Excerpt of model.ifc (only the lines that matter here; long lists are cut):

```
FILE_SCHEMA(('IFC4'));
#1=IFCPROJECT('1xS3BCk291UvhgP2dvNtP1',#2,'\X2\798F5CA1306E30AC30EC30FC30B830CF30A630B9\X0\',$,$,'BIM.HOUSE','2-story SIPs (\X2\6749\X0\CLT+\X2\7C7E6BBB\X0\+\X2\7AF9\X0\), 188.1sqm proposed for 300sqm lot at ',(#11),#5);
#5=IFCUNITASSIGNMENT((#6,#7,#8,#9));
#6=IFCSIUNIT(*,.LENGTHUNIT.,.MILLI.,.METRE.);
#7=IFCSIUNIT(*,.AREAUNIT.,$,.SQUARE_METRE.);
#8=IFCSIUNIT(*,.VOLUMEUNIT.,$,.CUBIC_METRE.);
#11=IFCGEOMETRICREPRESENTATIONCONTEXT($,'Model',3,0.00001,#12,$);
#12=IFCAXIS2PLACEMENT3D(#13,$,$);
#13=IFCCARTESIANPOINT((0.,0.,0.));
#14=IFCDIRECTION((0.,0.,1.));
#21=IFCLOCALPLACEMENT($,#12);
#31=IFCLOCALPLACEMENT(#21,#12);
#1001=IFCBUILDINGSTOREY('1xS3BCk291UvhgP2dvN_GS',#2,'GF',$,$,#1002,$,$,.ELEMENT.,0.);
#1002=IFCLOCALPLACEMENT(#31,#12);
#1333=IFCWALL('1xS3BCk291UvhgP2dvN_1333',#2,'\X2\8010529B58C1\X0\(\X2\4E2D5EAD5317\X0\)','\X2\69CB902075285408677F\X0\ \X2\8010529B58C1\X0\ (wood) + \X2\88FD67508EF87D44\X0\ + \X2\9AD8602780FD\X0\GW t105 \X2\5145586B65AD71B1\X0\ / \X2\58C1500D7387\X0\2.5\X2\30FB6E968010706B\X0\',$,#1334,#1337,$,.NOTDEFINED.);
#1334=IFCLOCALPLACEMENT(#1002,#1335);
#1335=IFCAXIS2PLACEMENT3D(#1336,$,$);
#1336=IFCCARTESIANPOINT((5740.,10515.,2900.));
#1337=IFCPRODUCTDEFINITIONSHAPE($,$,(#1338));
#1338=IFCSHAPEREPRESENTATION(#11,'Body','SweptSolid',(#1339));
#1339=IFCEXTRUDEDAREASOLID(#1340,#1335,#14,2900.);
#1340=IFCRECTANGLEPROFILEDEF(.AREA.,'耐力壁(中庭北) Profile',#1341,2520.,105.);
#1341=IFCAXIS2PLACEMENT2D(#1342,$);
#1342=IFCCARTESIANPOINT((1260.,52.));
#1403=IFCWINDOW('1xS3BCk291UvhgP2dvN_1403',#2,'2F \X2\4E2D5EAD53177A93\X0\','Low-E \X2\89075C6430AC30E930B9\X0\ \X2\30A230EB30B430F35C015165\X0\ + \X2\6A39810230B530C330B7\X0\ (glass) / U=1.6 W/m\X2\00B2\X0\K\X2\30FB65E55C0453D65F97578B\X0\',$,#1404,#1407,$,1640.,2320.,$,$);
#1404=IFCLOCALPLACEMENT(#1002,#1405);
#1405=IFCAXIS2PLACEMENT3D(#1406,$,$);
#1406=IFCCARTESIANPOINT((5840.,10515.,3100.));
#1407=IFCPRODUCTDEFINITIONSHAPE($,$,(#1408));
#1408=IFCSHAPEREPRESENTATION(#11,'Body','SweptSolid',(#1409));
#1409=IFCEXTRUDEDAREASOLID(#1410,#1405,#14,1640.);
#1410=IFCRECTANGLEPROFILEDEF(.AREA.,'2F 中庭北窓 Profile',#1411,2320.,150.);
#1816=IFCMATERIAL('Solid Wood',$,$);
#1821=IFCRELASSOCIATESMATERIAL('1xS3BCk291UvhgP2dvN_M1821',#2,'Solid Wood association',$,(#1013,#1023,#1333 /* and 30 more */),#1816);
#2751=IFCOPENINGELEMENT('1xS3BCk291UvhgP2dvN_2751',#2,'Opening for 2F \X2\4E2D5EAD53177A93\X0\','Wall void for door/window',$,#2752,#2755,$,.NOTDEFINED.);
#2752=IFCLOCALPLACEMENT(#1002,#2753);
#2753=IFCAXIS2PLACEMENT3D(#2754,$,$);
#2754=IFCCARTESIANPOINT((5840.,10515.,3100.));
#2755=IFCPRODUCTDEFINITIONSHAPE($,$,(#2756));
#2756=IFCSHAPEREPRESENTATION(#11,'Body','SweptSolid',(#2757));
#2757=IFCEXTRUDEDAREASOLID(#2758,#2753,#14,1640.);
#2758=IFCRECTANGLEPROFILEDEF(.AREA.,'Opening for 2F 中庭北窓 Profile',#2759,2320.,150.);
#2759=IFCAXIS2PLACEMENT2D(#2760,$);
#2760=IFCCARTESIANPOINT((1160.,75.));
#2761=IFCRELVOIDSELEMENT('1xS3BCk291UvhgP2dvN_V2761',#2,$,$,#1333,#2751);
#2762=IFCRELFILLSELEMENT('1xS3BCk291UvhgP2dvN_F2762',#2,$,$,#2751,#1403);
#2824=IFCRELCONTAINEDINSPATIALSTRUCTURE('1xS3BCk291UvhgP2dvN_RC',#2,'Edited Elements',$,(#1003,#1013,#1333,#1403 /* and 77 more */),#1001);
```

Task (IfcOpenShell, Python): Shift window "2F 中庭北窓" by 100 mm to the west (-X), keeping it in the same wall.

```python
import ifcopenshell
import ifcopenshell.api.geometry
import ifcopenshell.util.placement
import ifcopenshell.util.unit

model = ifcopenshell.open("model.ifc")
unit_scale = ifcopenshell.util.unit.calculate_unit_scale(model)

window = model.by_guid("1xS3BCk291UvhgP2dvN_1403")
opening = window.FillsVoids[0].RelatingOpeningElement
wall = opening.VoidsElements[0].RelatingBuildingElement

wall_matrix = ifcopenshell.util.placement.get_local_placement(wall.ObjectPlacement)
shift = wall_matrix[:3, 0] * -0.1 / unit_scale
before = ifcopenshell.util.placement.get_local_placement(window.ObjectPlacement)[:3, 3].copy()

# The window is not placed relative to its opening, so move both.
for product in (opening, window):
    matrix = ifcopenshell.util.placement.get_local_placement(product.ObjectPlacement)
    matrix[:3, 3] += shift
    ifcopenshell.api.geometry.edit_object_placement(model, product=product, matrix=matrix, is_si=False)

after = ifcopenshell.util.placement.get_local_placement(window.ObjectPlacement)[:3, 3]
print("window moved by", (after - before).round(3) + 0.0)

model.write("model-out.ifc")
```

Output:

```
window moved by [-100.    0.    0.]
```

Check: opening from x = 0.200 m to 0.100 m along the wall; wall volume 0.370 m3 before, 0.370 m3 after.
